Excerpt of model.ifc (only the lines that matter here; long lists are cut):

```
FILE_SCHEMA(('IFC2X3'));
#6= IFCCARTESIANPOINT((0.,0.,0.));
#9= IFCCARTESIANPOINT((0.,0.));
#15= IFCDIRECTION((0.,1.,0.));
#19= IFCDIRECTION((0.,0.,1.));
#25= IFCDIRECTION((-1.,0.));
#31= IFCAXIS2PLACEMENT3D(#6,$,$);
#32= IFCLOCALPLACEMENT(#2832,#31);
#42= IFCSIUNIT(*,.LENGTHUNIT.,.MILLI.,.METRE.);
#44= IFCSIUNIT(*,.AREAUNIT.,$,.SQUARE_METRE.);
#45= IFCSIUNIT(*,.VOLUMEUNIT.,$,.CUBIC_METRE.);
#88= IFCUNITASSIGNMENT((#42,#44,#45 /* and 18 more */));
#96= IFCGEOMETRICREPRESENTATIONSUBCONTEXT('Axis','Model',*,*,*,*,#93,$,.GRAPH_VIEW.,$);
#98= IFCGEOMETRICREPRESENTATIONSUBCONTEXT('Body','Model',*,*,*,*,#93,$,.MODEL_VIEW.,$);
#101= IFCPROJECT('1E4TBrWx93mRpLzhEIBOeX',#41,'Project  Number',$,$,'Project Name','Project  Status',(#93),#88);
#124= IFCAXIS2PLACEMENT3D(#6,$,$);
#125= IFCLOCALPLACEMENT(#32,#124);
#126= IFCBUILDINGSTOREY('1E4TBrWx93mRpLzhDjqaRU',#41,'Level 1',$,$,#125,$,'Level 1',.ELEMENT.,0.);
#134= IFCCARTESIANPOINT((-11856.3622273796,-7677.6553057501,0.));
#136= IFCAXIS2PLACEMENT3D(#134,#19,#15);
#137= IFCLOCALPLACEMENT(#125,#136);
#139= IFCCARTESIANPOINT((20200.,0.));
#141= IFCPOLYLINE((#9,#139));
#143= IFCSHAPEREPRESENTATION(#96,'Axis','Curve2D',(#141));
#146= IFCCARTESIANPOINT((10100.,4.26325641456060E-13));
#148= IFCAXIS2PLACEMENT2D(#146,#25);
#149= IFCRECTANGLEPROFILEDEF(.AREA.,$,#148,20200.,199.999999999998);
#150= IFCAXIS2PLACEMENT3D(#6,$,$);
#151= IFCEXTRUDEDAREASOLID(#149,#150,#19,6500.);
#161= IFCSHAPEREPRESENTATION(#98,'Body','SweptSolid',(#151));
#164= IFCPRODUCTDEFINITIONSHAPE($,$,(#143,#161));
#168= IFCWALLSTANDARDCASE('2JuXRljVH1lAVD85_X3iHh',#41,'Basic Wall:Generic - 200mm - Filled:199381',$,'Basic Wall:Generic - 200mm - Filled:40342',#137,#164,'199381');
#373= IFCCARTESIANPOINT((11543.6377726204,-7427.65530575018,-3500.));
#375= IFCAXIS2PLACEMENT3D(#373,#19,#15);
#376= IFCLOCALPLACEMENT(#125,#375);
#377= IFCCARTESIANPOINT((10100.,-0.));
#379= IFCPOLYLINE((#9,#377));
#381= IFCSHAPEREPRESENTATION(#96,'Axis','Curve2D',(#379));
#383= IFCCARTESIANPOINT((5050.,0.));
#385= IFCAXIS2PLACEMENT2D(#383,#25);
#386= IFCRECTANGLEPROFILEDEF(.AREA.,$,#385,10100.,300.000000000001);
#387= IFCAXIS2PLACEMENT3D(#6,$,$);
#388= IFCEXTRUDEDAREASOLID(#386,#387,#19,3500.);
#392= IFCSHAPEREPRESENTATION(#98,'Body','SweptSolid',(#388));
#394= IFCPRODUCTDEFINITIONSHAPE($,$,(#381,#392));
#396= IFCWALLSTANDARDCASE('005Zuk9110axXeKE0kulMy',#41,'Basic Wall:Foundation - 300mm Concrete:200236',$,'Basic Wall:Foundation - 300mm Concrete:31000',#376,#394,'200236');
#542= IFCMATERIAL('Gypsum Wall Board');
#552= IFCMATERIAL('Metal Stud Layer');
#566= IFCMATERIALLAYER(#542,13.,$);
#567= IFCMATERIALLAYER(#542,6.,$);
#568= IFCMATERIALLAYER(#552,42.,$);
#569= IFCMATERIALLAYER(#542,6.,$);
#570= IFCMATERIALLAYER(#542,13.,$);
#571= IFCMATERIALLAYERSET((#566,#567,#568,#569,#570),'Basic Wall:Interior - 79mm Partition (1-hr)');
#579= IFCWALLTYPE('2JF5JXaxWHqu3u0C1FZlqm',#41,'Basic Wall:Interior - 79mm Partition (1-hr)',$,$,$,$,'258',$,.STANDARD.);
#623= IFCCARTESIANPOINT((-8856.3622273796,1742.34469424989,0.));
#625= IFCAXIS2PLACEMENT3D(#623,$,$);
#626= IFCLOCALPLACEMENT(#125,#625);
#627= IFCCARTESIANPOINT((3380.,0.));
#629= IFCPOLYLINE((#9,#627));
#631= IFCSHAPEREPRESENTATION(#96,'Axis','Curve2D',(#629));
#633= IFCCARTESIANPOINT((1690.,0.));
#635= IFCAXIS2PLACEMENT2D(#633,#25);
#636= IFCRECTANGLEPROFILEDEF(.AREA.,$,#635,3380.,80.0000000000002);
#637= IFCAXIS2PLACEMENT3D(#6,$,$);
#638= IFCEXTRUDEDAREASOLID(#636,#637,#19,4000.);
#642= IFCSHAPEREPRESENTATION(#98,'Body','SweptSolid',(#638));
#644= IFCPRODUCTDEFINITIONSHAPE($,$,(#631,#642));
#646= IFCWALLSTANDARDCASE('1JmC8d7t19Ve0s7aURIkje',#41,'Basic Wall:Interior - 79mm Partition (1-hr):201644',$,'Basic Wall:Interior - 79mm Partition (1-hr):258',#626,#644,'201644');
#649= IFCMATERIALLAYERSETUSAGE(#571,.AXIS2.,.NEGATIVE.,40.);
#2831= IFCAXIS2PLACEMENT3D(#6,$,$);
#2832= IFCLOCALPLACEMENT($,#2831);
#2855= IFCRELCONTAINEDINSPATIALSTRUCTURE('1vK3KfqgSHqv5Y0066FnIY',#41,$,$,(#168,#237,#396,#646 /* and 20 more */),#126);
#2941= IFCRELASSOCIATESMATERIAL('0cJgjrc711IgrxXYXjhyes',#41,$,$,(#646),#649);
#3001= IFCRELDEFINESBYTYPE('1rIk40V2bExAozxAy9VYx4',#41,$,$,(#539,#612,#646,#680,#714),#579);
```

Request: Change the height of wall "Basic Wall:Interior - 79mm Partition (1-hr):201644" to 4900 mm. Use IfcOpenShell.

```python
import ifcopenshell
import ifcopenshell.geom
import ifcopenshell.util.representation
import ifcopenshell.util.shape
import ifcopenshell.util.unit

model = ifcopenshell.open("model.ifc")
unit_scale = ifcopenshell.util.unit.calculate_unit_scale(model)
settings = ifcopenshell.geom.settings()


def volume(element):
    """Net volume in cubic metres, openings subtracted."""
    shape = ifcopenshell.geom.create_shape(settings, element)
    return ifcopenshell.util.shape.get_volume(shape.geometry)


wall = model.by_guid("1JmC8d7t19Ve0s7aURIkje")
before = volume(wall)

body = ifcopenshell.util.representation.get_representation(wall, "Model", "Body")
solid = body.Items[0]
old_height = solid.Depth
solid.Depth = 4.9 / unit_scale
after = volume(wall)

print(f"height {old_height:g} -> {solid.Depth:g}, volume {before:.3f} -> {after:.3f} m3")

model.write("model_rev.ifc")
```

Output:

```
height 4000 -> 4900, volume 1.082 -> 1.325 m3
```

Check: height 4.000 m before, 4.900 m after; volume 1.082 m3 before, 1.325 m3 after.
